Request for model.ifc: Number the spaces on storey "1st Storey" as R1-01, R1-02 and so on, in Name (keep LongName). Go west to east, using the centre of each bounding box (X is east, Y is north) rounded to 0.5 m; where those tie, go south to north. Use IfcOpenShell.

First a look at what the model holds.

```python
import ifcopenshell
import ifcopenshell.util.element
import ifcopenshell.util.placement

model = ifcopenshell.open("model.ifc")
print(model.schema)
storey = next(s for s in model.by_type("IfcBuildingStorey") if s.Name == "1st Storey")
spaces = [e for e in ifcopenshell.util.element.get_decomposition(storey) if e.is_a("IfcSpace")]
for e in sorted(spaces, key=lambda e: e.id()):
    origin = ifcopenshell.util.placement.get_local_placement(e.ObjectPlacement)[:3, 3]
    print(e.id(), e.Name, e.LongName, origin.round(2) + 0.0, sep=" | ")
```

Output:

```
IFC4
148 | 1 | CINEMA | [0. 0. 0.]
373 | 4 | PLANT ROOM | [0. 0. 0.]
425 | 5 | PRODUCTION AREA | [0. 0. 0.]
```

```python
import ifcopenshell
import ifcopenshell.geom
import ifcopenshell.util.element
import ifcopenshell.util.shape

model = ifcopenshell.open("model.ifc")
settings = ifcopenshell.geom.settings()
settings.set("use-world-coords", True)


def centre(element):
    shape = ifcopenshell.geom.create_shape(settings, element)
    return ifcopenshell.util.shape.get_bbox_centroid(shape.geometry)


storey = next(s for s in model.by_type("IfcBuildingStorey") if s.Name == "1st Storey")
spaces = [e for e in ifcopenshell.util.element.get_decomposition(storey) if e.is_a("IfcSpace")]

# Insertion points can sit at a corner or the storey origin, so sort by the geometry (in metres).
centres = {e: centre(e) for e in spaces}
spaces.sort(key=lambda e: (round(centres[e][0] / 0.5), centres[e][1]))

for i, e in enumerate(spaces, start=1):
    number = f"R1-{i:02d}"
    e.Name = number
    print(e.id(), number)

model.write("model_edited.ifc")
```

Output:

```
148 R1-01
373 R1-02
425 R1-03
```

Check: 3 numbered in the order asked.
